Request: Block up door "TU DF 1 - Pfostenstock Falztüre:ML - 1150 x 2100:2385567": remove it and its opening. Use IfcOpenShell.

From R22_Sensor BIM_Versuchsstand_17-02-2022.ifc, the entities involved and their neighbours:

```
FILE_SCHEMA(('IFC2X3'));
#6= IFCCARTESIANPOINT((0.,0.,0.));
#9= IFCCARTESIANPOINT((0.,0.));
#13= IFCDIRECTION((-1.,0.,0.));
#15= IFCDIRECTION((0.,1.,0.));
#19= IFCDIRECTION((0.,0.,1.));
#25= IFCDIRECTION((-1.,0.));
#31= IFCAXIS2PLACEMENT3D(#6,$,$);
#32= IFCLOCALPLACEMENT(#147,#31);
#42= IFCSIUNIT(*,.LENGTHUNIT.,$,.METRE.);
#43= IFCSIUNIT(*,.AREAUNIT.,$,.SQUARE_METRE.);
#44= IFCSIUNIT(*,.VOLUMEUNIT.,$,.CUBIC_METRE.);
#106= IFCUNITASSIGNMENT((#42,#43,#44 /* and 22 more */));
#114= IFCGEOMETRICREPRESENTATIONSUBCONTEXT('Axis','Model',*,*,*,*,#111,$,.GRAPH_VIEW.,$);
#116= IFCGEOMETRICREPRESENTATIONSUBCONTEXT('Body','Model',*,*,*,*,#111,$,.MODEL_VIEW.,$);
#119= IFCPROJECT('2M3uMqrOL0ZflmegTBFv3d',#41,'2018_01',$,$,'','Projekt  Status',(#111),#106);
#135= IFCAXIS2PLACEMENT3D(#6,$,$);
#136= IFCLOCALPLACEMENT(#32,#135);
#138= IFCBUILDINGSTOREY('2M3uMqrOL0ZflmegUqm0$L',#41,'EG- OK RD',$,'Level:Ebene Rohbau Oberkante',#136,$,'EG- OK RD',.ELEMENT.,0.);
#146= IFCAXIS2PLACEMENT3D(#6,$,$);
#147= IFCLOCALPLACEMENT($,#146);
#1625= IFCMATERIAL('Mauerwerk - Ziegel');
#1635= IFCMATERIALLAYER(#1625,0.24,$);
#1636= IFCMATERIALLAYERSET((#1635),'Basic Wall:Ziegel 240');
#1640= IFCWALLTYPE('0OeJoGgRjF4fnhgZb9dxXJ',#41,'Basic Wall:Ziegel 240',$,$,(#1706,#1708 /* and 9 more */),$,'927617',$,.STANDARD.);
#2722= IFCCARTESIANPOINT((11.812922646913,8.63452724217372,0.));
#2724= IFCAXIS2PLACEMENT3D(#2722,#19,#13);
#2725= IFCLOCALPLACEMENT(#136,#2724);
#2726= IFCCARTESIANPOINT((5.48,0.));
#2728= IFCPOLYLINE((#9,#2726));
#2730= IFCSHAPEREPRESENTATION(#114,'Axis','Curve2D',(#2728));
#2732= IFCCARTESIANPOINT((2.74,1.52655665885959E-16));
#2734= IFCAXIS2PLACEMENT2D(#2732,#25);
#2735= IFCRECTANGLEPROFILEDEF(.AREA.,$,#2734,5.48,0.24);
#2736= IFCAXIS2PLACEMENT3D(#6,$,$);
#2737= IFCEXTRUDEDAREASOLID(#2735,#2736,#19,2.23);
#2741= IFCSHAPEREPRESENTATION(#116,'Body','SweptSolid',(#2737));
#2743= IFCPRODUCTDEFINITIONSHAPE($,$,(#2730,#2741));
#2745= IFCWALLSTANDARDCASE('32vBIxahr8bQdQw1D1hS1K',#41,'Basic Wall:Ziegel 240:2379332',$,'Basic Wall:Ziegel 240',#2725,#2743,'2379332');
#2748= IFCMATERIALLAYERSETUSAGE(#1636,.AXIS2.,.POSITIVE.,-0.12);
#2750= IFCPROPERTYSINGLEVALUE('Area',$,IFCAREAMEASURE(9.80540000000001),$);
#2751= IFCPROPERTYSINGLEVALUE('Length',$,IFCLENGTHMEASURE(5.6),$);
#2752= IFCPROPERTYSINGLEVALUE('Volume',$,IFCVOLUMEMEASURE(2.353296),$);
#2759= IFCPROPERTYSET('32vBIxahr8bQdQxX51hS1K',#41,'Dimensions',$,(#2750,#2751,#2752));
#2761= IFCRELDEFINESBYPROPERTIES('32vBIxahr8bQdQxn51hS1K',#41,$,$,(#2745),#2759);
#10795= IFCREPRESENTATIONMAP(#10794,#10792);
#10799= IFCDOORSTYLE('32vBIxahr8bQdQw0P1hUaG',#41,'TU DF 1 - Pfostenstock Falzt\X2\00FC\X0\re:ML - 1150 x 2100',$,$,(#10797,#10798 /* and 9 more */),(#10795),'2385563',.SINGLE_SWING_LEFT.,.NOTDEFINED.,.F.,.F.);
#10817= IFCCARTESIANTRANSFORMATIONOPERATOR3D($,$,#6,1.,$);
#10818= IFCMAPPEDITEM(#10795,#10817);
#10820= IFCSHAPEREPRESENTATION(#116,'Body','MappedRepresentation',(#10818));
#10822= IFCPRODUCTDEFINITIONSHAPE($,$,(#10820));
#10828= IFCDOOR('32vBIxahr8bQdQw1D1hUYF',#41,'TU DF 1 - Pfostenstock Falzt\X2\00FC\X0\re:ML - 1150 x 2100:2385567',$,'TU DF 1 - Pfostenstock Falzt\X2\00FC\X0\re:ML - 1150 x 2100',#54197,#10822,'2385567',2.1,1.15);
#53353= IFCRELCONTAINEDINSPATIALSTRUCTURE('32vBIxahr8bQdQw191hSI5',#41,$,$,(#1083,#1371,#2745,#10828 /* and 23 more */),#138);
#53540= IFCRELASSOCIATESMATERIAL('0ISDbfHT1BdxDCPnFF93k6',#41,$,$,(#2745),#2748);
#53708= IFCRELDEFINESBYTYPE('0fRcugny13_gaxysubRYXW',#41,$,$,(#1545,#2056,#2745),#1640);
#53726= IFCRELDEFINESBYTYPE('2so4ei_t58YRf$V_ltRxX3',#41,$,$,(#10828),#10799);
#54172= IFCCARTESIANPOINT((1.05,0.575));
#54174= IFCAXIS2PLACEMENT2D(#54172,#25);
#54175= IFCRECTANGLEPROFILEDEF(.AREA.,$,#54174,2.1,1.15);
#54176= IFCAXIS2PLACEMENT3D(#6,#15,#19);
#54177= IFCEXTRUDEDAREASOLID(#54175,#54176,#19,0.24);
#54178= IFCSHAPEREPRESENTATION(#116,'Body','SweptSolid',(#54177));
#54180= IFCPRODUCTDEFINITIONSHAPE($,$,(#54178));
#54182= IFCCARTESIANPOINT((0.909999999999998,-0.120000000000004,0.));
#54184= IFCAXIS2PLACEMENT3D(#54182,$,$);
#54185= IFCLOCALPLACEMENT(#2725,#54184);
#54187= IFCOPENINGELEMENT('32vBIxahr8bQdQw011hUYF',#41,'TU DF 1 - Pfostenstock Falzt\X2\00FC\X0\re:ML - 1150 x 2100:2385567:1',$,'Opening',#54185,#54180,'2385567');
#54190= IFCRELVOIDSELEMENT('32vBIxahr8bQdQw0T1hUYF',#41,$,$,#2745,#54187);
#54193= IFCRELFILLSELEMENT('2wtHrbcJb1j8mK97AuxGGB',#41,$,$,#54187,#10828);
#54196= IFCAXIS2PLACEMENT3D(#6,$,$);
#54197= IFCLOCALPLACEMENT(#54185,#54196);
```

```python
import ifcopenshell
import ifcopenshell.api.feature
import ifcopenshell.api.pset
import ifcopenshell.api.root
import ifcopenshell.geom
import ifcopenshell.util.element
import ifcopenshell.util.shape
import ifcopenshell.util.unit

model = ifcopenshell.open("R22_Sensor BIM_Versuchsstand_17-02-2022.ifc")
area_scale = ifcopenshell.util.unit.calculate_unit_scale(model, "AREAUNIT")
volume_scale = ifcopenshell.util.unit.calculate_unit_scale(model, "VOLUMEUNIT")
settings = ifcopenshell.geom.settings()


def volume(element):
    """Net volume in cubic metres, openings subtracted."""
    shape = ifcopenshell.geom.create_shape(settings, element)
    return ifcopenshell.util.shape.get_volume(shape.geometry)


door = model.by_id(10828)
opening = door.FillsVoids[0].RelatingOpeningElement
wall = opening.VoidsElements[0].RelatingBuildingElement
before = volume(wall)

ifcopenshell.api.root.remove_product(model, product=door)
ifcopenshell.api.feature.remove_feature(model, feature=opening)

after = volume(wall)
thickness = 0.24  # wall thickness in metres

# Update the wall's stored quantities.
pset = model.by_id(ifcopenshell.util.element.get_pset(wall, "Dimensions", should_inherit=False)["id"])
ifcopenshell.api.pset.edit_pset(model, pset=pset, properties={
    "Area": model.create_entity("IfcAreaMeasure", after / thickness / area_scale),
    "Volume": model.create_entity("IfcVolumeMeasure", after / volume_scale),
})

print(f"wall volume {before:.3f} -> {after:.3f} m3")

model.write("R22_Sensor BIM_Versuchsstand_17-02-2022_edited.ifc")
```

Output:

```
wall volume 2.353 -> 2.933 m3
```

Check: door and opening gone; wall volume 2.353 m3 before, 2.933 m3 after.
